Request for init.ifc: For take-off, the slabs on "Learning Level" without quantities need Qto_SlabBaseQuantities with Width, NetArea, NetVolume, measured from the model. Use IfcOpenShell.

First a look at what the model holds.

```python
import ifcopenshell
import ifcopenshell.util.element
import ifcopenshell.util.unit

model = ifcopenshell.open("init.ifc")
print(model.schema)
for unit_type in ("LENGTHUNIT", "AREAUNIT", "VOLUMEUNIT"):
    print(unit_type, ifcopenshell.util.unit.calculate_unit_scale(model, unit_type))
storey = next(s for s in model.by_type("IfcBuildingStorey") if s.Name == "Learning Level")
slabs = [e for e in ifcopenshell.util.element.get_decomposition(storey) if e.is_a("IfcSlab")]
for e in sorted(slabs, key=lambda e: e.id()):
    print(e.id(), e.is_a(), e.Name, list(ifcopenshell.util.element.get_psets(e, qtos_only=True)), sep=" | ")
```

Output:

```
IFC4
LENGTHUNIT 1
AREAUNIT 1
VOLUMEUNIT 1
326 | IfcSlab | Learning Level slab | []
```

```python
import ifcopenshell
import ifcopenshell.api.pset
import ifcopenshell.geom
import ifcopenshell.util.element
import ifcopenshell.util.shape
import ifcopenshell.util.unit

model = ifcopenshell.open("init.ifc")
unit_scale = ifcopenshell.util.unit.calculate_unit_scale(model)
area_scale = ifcopenshell.util.unit.calculate_unit_scale(model, "AREAUNIT")
volume_scale = ifcopenshell.util.unit.calculate_unit_scale(model, "VOLUMEUNIT")
settings = ifcopenshell.geom.settings()

storey = next(s for s in model.by_type("IfcBuildingStorey") if s.Name == "Learning Level")
slabs = [e for e in ifcopenshell.util.element.get_decomposition(storey) if e.is_a("IfcSlab")]

for e in sorted(slabs, key=lambda e: e.id()):
    if ifcopenshell.util.element.get_psets(e, qtos_only=True, should_inherit=False):
        continue
    # Geometry comes back in metres, in the element's own axes.
    shape = ifcopenshell.geom.create_shape(settings, e)
    values = {
        "Width": ifcopenshell.util.shape.get_z(shape.geometry) / unit_scale,
        "NetArea": ifcopenshell.util.shape.get_footprint_area(shape.geometry) / area_scale,
        "NetVolume": ifcopenshell.util.shape.get_volume(shape.geometry) / volume_scale,
    }
    qto = ifcopenshell.api.pset.add_qto(model, product=e, name="Qto_SlabBaseQuantities")
    ifcopenshell.api.pset.edit_qto(model, qto=qto, properties=values)
    print(e.id(), {k: round(v, 3) for k, v in values.items()})

model.write("init_updated.ifc")
```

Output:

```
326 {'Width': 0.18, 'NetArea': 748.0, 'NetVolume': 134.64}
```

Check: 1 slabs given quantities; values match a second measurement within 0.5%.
